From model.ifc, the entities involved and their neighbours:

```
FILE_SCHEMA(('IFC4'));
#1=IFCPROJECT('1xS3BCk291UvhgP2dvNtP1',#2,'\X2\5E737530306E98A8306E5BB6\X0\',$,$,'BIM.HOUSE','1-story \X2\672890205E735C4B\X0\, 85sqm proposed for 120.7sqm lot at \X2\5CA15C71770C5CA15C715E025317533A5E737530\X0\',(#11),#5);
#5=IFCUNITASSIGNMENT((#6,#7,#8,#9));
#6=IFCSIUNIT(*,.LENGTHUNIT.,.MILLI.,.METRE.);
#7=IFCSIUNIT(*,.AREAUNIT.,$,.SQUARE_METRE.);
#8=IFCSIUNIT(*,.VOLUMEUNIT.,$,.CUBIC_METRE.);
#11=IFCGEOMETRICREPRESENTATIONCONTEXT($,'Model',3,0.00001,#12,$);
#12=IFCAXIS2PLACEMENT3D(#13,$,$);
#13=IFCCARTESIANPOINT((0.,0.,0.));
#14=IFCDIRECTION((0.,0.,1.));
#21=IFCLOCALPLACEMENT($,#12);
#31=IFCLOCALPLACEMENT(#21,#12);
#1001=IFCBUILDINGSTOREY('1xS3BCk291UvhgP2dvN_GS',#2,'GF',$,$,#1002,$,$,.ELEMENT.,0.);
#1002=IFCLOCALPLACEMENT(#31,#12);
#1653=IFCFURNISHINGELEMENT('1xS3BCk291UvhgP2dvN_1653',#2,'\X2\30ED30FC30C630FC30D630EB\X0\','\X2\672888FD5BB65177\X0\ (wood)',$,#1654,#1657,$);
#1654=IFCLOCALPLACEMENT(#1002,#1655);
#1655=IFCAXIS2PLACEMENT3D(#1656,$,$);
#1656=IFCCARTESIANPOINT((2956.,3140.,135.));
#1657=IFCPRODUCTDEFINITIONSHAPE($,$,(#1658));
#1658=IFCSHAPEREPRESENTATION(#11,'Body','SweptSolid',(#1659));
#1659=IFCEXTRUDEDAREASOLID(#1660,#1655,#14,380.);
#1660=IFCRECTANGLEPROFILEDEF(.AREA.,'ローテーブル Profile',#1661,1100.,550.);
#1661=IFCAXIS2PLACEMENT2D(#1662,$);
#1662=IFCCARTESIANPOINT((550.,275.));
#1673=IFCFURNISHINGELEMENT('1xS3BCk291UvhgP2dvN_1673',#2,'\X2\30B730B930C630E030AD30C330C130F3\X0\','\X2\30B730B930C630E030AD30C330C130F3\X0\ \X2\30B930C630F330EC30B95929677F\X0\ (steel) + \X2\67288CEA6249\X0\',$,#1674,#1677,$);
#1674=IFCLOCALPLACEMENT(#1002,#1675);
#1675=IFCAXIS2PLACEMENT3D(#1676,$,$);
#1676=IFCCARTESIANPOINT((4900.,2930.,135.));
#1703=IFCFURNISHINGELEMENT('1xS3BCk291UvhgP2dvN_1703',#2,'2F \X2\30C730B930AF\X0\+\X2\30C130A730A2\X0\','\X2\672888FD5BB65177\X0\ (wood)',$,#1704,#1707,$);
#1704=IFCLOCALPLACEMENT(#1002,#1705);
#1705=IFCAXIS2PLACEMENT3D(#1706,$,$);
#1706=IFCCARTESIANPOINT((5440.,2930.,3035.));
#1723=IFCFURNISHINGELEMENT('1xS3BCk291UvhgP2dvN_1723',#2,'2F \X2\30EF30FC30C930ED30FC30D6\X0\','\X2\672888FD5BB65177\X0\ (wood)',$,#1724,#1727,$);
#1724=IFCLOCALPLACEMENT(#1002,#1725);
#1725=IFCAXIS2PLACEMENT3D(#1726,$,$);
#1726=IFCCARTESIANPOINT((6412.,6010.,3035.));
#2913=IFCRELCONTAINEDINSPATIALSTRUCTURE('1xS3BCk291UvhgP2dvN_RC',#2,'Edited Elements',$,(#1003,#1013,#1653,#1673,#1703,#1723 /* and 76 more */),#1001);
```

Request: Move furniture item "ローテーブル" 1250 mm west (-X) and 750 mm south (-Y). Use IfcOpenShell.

```python
import ifcopenshell
import ifcopenshell.api.geometry
import ifcopenshell.util.placement
import ifcopenshell.util.unit

model = ifcopenshell.open("model.ifc")
unit_scale = ifcopenshell.util.unit.calculate_unit_scale(model)

item = model.by_guid("1xS3BCk291UvhgP2dvN_1653")
matrix = ifcopenshell.util.placement.get_local_placement(item.ObjectPlacement)
matrix[0, 3] -= 1.25 / unit_scale
matrix[1, 3] -= 0.75 / unit_scale
ifcopenshell.api.geometry.edit_object_placement(model, product=item, matrix=matrix, is_si=False)

print(ifcopenshell.util.placement.get_local_placement(item.ObjectPlacement).round(3) + 0.0)

model.write("model_v2.ifc")
```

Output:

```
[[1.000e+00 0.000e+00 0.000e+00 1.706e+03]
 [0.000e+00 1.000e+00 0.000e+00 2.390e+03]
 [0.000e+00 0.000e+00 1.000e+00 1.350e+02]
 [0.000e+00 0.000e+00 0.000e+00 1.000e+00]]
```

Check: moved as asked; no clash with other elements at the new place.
